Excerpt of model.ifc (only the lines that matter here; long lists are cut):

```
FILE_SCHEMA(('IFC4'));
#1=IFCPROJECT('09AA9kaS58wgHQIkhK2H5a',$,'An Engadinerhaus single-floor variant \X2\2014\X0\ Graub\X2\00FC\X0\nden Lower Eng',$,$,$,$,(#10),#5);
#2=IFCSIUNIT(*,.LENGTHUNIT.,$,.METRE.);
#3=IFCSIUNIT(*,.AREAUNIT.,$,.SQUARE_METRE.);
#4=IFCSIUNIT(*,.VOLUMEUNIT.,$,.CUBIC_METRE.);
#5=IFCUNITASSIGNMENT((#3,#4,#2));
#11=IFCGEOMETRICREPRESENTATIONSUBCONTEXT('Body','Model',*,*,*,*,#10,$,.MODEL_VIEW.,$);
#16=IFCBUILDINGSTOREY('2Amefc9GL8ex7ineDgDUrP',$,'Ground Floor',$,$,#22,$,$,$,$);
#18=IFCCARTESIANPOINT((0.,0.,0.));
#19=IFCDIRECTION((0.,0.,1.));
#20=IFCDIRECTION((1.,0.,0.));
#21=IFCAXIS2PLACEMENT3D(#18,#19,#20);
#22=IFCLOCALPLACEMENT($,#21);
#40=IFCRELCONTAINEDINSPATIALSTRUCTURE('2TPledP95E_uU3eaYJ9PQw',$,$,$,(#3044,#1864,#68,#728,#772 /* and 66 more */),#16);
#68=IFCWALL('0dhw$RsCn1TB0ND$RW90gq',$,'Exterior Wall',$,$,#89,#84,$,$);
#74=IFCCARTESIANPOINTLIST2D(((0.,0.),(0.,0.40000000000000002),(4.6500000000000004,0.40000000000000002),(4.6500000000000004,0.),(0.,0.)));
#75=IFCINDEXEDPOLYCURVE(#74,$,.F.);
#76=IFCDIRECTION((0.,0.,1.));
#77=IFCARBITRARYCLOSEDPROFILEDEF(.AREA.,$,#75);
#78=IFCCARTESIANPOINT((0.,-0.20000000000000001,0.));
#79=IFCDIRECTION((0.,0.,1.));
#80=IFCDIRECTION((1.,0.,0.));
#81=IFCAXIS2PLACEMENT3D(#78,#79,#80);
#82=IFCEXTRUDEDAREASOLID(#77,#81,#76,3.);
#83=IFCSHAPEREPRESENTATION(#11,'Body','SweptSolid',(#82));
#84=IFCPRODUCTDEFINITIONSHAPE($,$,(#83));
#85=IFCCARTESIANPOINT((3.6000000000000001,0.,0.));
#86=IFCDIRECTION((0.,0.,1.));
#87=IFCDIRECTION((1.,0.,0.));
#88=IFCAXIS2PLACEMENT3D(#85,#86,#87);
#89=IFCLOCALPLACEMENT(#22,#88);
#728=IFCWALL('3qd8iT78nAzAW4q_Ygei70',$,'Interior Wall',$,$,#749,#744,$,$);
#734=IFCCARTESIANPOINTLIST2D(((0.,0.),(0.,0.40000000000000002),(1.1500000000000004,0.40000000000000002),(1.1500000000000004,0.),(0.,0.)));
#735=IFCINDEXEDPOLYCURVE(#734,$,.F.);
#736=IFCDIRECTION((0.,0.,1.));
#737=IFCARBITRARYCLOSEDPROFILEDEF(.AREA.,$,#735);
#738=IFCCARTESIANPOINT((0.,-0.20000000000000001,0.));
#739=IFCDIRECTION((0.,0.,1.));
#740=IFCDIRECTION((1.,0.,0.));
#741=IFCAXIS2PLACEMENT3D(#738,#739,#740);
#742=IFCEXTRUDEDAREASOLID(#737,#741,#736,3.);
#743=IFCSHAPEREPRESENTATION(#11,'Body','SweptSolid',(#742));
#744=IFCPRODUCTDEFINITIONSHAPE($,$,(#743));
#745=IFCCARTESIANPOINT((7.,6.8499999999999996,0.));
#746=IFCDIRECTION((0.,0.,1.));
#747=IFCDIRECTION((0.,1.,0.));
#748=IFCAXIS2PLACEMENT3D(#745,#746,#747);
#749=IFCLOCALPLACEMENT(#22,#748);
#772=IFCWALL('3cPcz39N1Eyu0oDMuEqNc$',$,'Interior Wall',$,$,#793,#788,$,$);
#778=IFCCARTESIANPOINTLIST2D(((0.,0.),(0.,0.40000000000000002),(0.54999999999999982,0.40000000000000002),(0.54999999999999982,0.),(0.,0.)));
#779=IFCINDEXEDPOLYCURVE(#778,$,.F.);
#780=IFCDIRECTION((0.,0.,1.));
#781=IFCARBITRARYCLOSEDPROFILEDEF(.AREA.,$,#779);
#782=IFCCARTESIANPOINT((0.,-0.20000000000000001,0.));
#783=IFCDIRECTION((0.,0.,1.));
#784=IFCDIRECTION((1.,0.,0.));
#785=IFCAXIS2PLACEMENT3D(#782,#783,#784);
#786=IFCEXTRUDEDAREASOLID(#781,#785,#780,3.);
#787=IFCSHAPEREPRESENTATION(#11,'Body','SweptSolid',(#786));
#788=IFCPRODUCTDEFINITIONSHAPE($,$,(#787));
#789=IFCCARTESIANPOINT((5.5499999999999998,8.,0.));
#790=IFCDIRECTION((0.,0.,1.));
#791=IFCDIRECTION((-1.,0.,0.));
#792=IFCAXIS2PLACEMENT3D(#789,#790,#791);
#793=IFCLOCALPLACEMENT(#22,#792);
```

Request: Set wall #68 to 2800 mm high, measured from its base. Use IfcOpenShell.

```python
import ifcopenshell
import ifcopenshell.geom
import ifcopenshell.util.representation
import ifcopenshell.util.shape

model = ifcopenshell.open("model.ifc")
settings = ifcopenshell.geom.settings()


def volume(element):
    """Net volume in cubic metres, openings subtracted."""
    shape = ifcopenshell.geom.create_shape(settings, element)
    return ifcopenshell.util.shape.get_volume(shape.geometry)


wall = model.by_id(68)
before = volume(wall)

body = ifcopenshell.util.representation.get_representation(wall, "Model", "Body")
solid = body.Items[0]
old_height = solid.Depth
solid.Depth = 2.8
after = volume(wall)

print(f"height {old_height:g} -> {solid.Depth:g}, volume {before:.3f} -> {after:.3f} m3")

model.write("model_edited.ifc")
```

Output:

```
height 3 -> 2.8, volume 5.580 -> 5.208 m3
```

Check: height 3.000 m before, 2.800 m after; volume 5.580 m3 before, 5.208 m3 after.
